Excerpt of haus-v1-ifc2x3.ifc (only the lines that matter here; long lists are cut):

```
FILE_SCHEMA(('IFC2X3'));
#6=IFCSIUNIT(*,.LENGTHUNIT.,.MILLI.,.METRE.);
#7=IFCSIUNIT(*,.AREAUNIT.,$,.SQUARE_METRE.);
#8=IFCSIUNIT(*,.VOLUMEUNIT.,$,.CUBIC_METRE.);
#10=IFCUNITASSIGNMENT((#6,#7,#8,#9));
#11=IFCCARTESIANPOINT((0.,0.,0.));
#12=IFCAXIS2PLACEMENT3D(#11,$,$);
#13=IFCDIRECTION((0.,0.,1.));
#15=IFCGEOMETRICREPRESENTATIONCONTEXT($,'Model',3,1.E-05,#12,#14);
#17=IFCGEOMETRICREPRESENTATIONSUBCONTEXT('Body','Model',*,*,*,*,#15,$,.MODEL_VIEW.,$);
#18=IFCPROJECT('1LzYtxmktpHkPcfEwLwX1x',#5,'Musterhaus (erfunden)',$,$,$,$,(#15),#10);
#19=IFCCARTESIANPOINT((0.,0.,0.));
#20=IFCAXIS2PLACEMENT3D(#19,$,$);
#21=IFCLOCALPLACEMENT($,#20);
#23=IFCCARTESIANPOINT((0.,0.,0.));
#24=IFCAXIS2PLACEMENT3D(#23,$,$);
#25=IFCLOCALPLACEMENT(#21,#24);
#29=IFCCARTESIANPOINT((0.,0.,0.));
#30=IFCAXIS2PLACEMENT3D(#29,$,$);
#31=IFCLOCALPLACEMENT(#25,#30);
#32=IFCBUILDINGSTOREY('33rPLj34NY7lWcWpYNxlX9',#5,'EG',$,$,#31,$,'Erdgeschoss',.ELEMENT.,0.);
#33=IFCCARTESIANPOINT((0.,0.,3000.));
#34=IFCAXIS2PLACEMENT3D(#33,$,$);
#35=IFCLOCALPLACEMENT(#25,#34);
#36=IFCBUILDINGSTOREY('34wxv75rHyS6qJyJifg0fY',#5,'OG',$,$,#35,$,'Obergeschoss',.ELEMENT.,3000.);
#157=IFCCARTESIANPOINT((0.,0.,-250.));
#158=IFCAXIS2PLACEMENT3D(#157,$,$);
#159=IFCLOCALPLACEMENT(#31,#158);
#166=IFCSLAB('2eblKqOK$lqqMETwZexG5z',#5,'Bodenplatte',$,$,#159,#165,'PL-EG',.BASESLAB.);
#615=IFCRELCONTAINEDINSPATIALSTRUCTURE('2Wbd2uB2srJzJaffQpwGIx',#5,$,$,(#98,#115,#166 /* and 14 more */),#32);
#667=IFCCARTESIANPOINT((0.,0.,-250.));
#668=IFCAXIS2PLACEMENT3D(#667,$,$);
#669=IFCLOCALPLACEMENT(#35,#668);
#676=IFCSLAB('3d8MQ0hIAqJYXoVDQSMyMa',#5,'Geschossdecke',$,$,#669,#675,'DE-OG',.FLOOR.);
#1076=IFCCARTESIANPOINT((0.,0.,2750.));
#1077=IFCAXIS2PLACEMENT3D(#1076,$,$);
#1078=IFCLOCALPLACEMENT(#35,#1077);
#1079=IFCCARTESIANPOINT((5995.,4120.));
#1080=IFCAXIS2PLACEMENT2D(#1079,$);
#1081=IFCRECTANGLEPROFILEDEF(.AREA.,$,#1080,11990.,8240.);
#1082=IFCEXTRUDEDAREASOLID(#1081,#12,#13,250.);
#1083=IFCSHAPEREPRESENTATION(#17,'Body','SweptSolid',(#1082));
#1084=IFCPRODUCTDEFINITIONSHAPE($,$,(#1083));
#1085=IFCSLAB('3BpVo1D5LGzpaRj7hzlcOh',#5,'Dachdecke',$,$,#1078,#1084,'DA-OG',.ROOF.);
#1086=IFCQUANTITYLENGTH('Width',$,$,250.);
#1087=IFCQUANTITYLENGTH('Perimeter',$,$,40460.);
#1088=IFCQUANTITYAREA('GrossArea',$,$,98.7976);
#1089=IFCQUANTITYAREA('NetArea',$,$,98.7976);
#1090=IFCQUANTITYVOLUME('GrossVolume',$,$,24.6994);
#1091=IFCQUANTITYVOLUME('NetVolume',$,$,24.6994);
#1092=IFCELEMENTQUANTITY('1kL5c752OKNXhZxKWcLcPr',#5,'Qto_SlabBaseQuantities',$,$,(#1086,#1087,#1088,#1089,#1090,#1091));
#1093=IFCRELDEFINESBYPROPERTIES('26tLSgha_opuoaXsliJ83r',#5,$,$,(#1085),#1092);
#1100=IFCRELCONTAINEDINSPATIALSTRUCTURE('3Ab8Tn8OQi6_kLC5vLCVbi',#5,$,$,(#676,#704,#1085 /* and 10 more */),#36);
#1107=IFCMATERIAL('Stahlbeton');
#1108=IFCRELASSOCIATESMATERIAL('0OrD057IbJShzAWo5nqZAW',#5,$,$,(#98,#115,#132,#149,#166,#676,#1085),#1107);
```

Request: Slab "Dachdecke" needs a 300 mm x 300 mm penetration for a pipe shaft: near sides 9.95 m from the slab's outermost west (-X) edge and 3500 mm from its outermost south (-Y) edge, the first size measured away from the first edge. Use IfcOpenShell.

```python
import numpy as np
import ifcopenshell
import ifcopenshell.api.feature
import ifcopenshell.api.geometry
import ifcopenshell.api.pset
import ifcopenshell.api.root
import ifcopenshell.geom
import ifcopenshell.util.element
import ifcopenshell.util.placement
import ifcopenshell.util.representation
import ifcopenshell.util.shape
import ifcopenshell.util.unit

model = ifcopenshell.open("haus-v1-ifc2x3.ifc")
unit_scale = ifcopenshell.util.unit.calculate_unit_scale(model)
area_scale = ifcopenshell.util.unit.calculate_unit_scale(model, "AREAUNIT")
volume_scale = ifcopenshell.util.unit.calculate_unit_scale(model, "VOLUMEUNIT")
settings = ifcopenshell.geom.settings()


def volume(element):
    """Net volume in cubic metres, openings subtracted."""
    shape = ifcopenshell.geom.create_shape(settings, element)
    return ifcopenshell.util.shape.get_volume(shape.geometry)


slab = model.by_guid("3BpVo1D5LGzpaRj7hzlcOh")
before = volume(slab)

# Extent in the slab's own axes, in metres. The edges named are its -X and -Y sides.
slab_shape = ifcopenshell.geom.create_shape(settings, slab)
vertices = ifcopenshell.util.shape.get_vertices(slab_shape.geometry)
x_min, y_min, bottom = vertices.min(axis=0)
top = vertices[:, 2].max()

opening = ifcopenshell.api.root.create_entity(model, ifc_class="IfcOpeningElement", name="Pipe shaft opening")
context = ifcopenshell.util.representation.get_context(model, "Model", "Body", "MODEL_VIEW")
width, depth = 0.3, 0.3
outline = [(0.0, 0.0), (width, 0.0), (width, depth), (0.0, depth), (0.0, 0.0)]
# Overshoot both faces by 50 mm so the cut is clean.
shape = ifcopenshell.api.geometry.add_slab_representation(
    model, context=context, depth=top - bottom + 0.1, polyline=outline
)
ifcopenshell.api.geometry.assign_representation(model, product=opening, representation=shape)

matrix = ifcopenshell.util.placement.get_local_placement(slab.ObjectPlacement)
matrix[:, 3] = matrix @ np.append(np.array([x_min + 9.95, y_min + 3.5, bottom - 0.05]) / unit_scale, 1.0)
ifcopenshell.api.geometry.edit_object_placement(model, product=opening, matrix=matrix, is_si=False)
ifcopenshell.api.feature.add_feature(model, feature=opening, element=slab)

after = volume(slab)

# Update the slab's stored quantities.
qto = model.by_id(ifcopenshell.util.element.get_pset(slab, "Qto_SlabBaseQuantities", should_inherit=False)["id"])
ifcopenshell.api.pset.edit_qto(model, qto=qto, properties={
    "NetArea": after / (top - bottom) / area_scale,
    "NetVolume": after / volume_scale,
})

print(f"slab volume {before:.3f} -> {after:.3f} m3")

model.write("haus-v1-ifc2x3_v2.ifc")
```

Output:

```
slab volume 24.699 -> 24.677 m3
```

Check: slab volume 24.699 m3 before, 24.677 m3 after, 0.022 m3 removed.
